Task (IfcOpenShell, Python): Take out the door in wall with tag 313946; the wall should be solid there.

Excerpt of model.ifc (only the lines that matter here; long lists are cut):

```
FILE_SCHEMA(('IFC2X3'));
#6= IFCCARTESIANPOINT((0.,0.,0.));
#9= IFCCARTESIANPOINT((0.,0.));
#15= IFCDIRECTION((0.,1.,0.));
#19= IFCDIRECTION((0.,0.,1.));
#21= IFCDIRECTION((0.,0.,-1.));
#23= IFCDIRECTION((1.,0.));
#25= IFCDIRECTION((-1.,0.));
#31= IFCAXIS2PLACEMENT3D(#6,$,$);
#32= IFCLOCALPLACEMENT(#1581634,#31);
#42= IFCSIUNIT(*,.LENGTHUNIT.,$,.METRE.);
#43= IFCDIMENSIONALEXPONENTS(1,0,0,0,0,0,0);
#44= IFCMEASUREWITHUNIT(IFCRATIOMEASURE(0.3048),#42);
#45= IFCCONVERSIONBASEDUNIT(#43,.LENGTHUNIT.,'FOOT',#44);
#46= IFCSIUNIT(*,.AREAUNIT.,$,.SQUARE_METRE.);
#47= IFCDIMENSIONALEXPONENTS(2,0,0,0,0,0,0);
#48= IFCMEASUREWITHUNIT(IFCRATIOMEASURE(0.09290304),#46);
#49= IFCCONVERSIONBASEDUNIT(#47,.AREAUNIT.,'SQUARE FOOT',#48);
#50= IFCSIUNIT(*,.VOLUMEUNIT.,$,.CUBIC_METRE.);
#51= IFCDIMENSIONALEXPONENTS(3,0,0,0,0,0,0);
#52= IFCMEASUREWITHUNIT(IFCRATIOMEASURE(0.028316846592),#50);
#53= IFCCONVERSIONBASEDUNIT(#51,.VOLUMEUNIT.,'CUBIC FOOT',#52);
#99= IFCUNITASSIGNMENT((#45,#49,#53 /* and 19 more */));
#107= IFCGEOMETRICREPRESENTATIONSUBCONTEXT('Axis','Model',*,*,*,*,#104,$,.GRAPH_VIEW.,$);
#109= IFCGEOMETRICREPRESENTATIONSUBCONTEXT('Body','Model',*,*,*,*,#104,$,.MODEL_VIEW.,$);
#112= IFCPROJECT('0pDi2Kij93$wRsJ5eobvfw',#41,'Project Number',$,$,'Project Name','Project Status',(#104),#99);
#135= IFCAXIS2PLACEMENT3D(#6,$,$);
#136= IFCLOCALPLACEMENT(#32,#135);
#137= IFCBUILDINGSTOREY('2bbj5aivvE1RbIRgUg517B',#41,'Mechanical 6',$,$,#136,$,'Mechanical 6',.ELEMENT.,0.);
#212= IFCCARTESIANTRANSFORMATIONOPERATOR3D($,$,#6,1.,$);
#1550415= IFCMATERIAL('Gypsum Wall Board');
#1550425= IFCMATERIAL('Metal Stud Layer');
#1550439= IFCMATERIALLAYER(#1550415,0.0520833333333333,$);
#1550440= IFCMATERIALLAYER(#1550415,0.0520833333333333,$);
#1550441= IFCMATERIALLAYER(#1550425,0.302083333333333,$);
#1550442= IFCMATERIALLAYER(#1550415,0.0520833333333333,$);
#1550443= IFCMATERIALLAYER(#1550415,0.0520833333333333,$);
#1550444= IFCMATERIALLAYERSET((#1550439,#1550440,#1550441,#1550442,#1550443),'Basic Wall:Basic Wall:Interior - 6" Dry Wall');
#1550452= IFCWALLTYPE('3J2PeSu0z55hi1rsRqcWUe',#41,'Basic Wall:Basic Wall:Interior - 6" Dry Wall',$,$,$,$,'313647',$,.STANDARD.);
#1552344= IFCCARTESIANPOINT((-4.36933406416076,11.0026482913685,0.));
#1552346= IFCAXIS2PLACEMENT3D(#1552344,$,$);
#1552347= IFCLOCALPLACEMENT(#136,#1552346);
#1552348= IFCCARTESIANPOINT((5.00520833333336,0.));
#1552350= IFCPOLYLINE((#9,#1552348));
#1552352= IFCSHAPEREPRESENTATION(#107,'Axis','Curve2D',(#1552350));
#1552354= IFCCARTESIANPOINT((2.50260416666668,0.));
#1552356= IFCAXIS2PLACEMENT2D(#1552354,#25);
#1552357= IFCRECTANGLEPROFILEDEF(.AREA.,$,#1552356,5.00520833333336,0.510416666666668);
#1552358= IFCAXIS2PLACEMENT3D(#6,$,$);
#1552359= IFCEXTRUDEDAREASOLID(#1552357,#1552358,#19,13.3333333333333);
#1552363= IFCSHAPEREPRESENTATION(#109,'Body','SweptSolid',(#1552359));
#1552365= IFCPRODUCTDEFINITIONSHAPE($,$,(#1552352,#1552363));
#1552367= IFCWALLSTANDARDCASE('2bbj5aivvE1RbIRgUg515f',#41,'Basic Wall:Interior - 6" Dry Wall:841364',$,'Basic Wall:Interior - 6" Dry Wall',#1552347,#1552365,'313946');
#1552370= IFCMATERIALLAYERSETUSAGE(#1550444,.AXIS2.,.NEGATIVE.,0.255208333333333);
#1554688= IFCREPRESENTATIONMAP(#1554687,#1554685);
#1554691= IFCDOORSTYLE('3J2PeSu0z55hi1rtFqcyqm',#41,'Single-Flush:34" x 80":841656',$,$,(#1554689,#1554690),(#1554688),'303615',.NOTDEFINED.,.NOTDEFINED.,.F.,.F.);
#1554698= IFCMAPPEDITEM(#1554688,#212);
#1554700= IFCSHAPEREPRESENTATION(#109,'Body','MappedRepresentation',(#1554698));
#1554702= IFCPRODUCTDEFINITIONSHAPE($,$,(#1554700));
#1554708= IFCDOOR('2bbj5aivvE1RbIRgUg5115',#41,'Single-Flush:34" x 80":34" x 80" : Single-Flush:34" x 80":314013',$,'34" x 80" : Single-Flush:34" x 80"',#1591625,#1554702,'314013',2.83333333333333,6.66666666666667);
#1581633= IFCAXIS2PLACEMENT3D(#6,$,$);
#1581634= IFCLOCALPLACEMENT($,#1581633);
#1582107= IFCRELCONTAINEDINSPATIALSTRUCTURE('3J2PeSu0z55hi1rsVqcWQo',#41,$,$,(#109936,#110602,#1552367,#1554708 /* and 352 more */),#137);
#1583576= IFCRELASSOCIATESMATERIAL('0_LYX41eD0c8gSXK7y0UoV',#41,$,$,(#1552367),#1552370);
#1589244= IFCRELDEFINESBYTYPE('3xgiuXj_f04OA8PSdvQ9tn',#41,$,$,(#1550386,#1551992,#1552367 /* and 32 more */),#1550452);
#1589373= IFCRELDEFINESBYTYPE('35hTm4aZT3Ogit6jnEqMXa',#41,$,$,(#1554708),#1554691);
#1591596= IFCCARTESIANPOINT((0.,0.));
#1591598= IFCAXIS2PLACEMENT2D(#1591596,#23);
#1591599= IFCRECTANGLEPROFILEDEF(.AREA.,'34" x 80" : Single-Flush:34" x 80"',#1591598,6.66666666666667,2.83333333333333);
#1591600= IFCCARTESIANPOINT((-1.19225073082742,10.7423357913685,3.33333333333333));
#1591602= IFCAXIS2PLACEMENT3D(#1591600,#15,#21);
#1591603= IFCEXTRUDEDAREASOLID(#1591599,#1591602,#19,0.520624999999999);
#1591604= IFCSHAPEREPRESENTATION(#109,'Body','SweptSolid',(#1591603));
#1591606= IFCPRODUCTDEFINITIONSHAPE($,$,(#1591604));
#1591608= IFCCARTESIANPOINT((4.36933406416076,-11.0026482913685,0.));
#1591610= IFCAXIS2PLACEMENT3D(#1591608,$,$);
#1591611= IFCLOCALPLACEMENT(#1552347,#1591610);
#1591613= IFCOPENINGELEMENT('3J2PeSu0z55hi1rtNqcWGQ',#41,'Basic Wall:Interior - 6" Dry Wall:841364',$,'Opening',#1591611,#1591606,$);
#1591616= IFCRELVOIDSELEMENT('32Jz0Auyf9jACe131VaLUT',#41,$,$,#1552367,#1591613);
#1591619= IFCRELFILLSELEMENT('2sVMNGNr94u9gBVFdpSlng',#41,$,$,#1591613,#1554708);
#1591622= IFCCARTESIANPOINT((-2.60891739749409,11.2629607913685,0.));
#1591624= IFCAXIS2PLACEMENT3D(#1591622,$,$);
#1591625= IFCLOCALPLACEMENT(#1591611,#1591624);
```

```python
import ifcopenshell
import ifcopenshell.api.feature
import ifcopenshell.api.root
import ifcopenshell.geom
import ifcopenshell.util.shape

model = ifcopenshell.open("model.ifc")
settings = ifcopenshell.geom.settings()


def volume(element):
    """Net volume in cubic metres, openings subtracted."""
    shape = ifcopenshell.geom.create_shape(settings, element)
    return ifcopenshell.util.shape.get_volume(shape.geometry)


door = model.by_id(1554708)
opening = door.FillsVoids[0].RelatingOpeningElement
wall = opening.VoidsElements[0].RelatingBuildingElement
before = volume(wall)

ifcopenshell.api.root.remove_product(model, product=door)
ifcopenshell.api.feature.remove_feature(model, feature=opening)

after = volume(wall)

print(f"wall volume {before:.3f} -> {after:.3f} m3")

model.write("model-out.ifc")
```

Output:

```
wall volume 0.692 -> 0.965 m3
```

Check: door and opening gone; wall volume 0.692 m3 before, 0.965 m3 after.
